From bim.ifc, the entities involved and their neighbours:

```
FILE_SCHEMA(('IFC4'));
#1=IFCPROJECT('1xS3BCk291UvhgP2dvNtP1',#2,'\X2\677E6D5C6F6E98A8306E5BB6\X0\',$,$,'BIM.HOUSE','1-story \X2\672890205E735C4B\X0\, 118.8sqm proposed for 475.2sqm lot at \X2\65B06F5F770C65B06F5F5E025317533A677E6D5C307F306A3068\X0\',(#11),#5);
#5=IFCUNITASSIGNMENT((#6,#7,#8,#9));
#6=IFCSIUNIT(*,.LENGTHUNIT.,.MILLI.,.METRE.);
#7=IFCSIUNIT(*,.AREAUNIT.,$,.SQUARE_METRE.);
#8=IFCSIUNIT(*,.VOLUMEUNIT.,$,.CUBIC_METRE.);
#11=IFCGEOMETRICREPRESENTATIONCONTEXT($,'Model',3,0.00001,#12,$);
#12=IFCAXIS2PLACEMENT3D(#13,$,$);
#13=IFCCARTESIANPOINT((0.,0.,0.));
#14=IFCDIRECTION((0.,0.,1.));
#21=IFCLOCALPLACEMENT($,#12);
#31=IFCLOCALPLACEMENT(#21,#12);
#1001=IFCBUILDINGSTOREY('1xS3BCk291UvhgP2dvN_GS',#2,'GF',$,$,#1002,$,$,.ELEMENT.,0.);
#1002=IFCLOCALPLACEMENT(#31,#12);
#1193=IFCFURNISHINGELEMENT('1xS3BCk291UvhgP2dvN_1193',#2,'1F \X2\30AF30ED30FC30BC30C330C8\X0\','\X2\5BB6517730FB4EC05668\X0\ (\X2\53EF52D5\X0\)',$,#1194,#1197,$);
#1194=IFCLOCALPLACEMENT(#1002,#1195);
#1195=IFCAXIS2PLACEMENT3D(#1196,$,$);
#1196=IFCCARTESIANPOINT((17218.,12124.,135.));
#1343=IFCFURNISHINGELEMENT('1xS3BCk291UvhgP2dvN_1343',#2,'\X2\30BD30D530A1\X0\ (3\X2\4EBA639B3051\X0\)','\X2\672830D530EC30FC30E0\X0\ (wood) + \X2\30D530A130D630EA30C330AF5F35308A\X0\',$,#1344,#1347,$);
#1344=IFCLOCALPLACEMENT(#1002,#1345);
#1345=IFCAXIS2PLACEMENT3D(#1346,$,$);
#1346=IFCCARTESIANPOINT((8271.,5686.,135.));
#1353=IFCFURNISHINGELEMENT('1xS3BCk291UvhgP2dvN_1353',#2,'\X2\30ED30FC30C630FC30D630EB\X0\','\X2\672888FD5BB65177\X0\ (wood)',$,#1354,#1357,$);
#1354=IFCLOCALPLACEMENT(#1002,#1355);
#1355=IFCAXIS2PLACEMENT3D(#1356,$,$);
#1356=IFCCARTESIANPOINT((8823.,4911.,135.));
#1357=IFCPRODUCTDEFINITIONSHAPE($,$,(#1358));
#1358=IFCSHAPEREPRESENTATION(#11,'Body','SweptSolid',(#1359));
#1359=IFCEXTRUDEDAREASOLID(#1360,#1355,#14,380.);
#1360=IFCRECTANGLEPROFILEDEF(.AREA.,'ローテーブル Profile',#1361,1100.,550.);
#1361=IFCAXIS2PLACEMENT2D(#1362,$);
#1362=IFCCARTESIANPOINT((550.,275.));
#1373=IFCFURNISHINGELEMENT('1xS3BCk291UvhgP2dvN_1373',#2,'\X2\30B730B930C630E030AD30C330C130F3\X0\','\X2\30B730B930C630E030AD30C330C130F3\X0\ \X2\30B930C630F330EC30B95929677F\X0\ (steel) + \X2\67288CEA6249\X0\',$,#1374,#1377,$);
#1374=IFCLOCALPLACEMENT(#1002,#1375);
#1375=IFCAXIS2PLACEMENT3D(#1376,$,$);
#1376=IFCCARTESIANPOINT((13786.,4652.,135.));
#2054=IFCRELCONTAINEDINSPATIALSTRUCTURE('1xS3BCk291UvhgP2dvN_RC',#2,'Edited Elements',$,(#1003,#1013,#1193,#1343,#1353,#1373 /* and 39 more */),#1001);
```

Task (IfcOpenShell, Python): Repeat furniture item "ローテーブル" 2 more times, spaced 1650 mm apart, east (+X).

```python
import numpy as np
import ifcopenshell
import ifcopenshell.api.geometry
import ifcopenshell.api.root
import ifcopenshell.util.element
import ifcopenshell.util.placement

model = ifcopenshell.open("bim.ifc")


def reuse_history(source, copy):
    """copy_class also copies each property set's owner history, people and application; keep the originals."""
    for rel in copy.IsDefinedBy:
        if rel.is_a("IfcRelDefinesByProperties") and (history := rel.RelatingPropertyDefinition.OwnerHistory):
            rel.RelatingPropertyDefinition.OwnerHistory = source.OwnerHistory
            ifcopenshell.util.element.remove_deep2(model, history)


source = model.by_guid("1xS3BCk291UvhgP2dvN_1353")
base = ifcopenshell.util.placement.get_local_placement(source.ObjectPlacement)
step = np.array([1.0, 0.0, 0.0]) * 1650.0

for i in range(1, 3):
    copy = ifcopenshell.api.root.copy_class(model, product=source)
    copy.Representation = ifcopenshell.util.element.copy_deep(
        model, source.Representation, exclude=["IfcGeometricRepresentationContext", "IfcRepresentationMap"]
    )
    reuse_history(source, copy)
    matrix = base.copy()
    matrix[:3, 3] += i * step
    print("added at", matrix[:3, 3].round(3) + 0.0)
    ifcopenshell.api.geometry.edit_object_placement(model, product=copy, matrix=matrix, is_si=False)

model.write("bim-out.ifc")
```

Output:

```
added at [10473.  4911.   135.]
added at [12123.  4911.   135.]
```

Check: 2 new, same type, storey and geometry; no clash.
